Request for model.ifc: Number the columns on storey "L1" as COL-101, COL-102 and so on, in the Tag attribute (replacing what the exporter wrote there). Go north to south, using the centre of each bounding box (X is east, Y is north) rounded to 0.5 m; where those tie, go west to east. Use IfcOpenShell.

First a look at what the model holds.

```python
import ifcopenshell
import ifcopenshell.util.element
import ifcopenshell.util.placement

model = ifcopenshell.open("model.ifc")
print(model.schema)
storey = next(s for s in model.by_type("IfcBuildingStorey") if s.Name == "L1")
columns = [e for e in ifcopenshell.util.element.get_decomposition(storey) if e.is_a("IfcColumn")]
for e in sorted(columns, key=lambda e: e.id()):
    origin = ifcopenshell.util.placement.get_local_placement(e.ObjectPlacement)[:3, 3]
    print(e.id(), e.Tag, e.Name, origin.round(2) + 0.0, sep=" | ")
```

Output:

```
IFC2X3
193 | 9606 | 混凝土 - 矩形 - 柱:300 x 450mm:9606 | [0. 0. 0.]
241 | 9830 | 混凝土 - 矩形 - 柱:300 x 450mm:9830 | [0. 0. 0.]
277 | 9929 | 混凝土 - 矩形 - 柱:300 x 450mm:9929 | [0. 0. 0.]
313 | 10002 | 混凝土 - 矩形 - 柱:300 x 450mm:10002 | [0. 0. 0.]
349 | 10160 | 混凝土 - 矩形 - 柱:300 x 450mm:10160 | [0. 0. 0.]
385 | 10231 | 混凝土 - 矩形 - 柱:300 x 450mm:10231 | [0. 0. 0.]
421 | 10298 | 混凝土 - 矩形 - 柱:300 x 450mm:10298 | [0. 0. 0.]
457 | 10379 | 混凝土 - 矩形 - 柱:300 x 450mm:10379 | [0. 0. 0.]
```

```python
import ifcopenshell
import ifcopenshell.geom
import ifcopenshell.util.element
import ifcopenshell.util.shape

model = ifcopenshell.open("model.ifc")
settings = ifcopenshell.geom.settings()
settings.set("use-world-coords", True)


def centre(element):
    shape = ifcopenshell.geom.create_shape(settings, element)
    return ifcopenshell.util.shape.get_bbox_centroid(shape.geometry)


storey = next(s for s in model.by_type("IfcBuildingStorey") if s.Name == "L1")
columns = [e for e in ifcopenshell.util.element.get_decomposition(storey) if e.is_a("IfcColumn")]

# Insertion points can sit at a corner or the storey origin, so sort by the geometry (in metres).
centres = {e: centre(e) for e in columns}
columns.sort(key=lambda e: (-round(centres[e][1] / 0.5), centres[e][0]))

for i, e in enumerate(columns, start=1):
    number = f"COL-1{i:02d}"
    e.Tag = number
    print(e.id(), number)

model.write("model_updated.ifc")
```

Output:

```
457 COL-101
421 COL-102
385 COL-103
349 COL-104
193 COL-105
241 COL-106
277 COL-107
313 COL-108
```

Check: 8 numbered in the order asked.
